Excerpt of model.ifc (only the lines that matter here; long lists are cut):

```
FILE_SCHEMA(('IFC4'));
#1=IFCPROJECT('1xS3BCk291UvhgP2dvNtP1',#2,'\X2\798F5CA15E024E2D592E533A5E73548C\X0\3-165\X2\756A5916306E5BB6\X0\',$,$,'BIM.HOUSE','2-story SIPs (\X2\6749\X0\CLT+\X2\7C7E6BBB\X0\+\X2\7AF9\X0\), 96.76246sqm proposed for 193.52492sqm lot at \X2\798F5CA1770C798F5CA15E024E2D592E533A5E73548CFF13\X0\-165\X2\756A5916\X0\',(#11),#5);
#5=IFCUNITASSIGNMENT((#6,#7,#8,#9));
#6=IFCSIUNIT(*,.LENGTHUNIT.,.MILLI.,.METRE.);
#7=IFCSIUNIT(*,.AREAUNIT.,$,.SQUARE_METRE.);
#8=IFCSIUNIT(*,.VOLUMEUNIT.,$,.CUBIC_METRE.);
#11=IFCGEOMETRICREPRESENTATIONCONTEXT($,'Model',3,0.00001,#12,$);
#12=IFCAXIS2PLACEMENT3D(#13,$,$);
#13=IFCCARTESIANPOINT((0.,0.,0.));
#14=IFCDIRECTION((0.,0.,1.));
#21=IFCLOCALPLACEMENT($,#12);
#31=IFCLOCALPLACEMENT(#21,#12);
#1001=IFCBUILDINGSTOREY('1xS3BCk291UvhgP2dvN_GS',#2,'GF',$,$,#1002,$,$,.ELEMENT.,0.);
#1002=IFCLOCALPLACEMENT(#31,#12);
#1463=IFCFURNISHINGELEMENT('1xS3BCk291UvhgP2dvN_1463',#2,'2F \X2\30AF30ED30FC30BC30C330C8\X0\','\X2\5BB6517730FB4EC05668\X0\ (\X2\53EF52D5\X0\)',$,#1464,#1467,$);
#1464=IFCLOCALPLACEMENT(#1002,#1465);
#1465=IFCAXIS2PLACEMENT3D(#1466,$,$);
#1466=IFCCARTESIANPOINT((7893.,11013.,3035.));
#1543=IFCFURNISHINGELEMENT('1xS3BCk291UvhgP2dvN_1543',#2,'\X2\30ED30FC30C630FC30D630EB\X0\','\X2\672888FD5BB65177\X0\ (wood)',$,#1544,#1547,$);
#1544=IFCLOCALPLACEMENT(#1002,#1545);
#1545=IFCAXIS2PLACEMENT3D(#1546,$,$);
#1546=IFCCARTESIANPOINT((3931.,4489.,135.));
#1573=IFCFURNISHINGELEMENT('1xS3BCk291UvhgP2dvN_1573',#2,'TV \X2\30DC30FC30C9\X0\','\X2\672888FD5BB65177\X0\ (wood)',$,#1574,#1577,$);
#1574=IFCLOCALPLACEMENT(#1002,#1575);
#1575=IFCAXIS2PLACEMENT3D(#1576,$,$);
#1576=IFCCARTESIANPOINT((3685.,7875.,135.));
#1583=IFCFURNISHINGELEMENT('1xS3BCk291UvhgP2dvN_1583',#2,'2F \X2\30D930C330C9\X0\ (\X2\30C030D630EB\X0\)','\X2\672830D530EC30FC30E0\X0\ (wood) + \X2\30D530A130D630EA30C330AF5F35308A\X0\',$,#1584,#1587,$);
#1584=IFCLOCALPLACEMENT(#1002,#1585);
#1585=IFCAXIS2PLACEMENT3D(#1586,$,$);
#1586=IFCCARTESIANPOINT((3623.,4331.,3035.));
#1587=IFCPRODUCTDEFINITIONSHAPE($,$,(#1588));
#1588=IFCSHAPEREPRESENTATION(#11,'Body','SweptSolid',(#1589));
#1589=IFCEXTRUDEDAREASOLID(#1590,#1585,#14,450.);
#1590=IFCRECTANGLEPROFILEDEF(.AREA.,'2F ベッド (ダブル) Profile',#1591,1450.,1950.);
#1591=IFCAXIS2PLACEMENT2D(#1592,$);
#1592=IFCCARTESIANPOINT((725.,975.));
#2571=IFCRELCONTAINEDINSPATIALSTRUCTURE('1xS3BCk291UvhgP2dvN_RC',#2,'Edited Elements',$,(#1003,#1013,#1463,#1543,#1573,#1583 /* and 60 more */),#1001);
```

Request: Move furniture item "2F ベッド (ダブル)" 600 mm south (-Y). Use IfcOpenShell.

```python
import ifcopenshell
import ifcopenshell.api.geometry
import ifcopenshell.util.placement
import ifcopenshell.util.unit

model = ifcopenshell.open("model.ifc")
unit_scale = ifcopenshell.util.unit.calculate_unit_scale(model)

item = model.by_guid("1xS3BCk291UvhgP2dvN_1583")
matrix = ifcopenshell.util.placement.get_local_placement(item.ObjectPlacement)
matrix[1, 3] -= 0.6 / unit_scale
ifcopenshell.api.geometry.edit_object_placement(model, product=item, matrix=matrix, is_si=False)

print(ifcopenshell.util.placement.get_local_placement(item.ObjectPlacement).round(3) + 0.0)

model.write("model_rev.ifc")
```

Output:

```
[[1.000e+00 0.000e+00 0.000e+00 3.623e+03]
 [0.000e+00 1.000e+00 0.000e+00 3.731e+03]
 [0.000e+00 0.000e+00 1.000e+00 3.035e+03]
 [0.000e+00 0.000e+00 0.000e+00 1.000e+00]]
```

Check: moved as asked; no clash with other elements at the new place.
